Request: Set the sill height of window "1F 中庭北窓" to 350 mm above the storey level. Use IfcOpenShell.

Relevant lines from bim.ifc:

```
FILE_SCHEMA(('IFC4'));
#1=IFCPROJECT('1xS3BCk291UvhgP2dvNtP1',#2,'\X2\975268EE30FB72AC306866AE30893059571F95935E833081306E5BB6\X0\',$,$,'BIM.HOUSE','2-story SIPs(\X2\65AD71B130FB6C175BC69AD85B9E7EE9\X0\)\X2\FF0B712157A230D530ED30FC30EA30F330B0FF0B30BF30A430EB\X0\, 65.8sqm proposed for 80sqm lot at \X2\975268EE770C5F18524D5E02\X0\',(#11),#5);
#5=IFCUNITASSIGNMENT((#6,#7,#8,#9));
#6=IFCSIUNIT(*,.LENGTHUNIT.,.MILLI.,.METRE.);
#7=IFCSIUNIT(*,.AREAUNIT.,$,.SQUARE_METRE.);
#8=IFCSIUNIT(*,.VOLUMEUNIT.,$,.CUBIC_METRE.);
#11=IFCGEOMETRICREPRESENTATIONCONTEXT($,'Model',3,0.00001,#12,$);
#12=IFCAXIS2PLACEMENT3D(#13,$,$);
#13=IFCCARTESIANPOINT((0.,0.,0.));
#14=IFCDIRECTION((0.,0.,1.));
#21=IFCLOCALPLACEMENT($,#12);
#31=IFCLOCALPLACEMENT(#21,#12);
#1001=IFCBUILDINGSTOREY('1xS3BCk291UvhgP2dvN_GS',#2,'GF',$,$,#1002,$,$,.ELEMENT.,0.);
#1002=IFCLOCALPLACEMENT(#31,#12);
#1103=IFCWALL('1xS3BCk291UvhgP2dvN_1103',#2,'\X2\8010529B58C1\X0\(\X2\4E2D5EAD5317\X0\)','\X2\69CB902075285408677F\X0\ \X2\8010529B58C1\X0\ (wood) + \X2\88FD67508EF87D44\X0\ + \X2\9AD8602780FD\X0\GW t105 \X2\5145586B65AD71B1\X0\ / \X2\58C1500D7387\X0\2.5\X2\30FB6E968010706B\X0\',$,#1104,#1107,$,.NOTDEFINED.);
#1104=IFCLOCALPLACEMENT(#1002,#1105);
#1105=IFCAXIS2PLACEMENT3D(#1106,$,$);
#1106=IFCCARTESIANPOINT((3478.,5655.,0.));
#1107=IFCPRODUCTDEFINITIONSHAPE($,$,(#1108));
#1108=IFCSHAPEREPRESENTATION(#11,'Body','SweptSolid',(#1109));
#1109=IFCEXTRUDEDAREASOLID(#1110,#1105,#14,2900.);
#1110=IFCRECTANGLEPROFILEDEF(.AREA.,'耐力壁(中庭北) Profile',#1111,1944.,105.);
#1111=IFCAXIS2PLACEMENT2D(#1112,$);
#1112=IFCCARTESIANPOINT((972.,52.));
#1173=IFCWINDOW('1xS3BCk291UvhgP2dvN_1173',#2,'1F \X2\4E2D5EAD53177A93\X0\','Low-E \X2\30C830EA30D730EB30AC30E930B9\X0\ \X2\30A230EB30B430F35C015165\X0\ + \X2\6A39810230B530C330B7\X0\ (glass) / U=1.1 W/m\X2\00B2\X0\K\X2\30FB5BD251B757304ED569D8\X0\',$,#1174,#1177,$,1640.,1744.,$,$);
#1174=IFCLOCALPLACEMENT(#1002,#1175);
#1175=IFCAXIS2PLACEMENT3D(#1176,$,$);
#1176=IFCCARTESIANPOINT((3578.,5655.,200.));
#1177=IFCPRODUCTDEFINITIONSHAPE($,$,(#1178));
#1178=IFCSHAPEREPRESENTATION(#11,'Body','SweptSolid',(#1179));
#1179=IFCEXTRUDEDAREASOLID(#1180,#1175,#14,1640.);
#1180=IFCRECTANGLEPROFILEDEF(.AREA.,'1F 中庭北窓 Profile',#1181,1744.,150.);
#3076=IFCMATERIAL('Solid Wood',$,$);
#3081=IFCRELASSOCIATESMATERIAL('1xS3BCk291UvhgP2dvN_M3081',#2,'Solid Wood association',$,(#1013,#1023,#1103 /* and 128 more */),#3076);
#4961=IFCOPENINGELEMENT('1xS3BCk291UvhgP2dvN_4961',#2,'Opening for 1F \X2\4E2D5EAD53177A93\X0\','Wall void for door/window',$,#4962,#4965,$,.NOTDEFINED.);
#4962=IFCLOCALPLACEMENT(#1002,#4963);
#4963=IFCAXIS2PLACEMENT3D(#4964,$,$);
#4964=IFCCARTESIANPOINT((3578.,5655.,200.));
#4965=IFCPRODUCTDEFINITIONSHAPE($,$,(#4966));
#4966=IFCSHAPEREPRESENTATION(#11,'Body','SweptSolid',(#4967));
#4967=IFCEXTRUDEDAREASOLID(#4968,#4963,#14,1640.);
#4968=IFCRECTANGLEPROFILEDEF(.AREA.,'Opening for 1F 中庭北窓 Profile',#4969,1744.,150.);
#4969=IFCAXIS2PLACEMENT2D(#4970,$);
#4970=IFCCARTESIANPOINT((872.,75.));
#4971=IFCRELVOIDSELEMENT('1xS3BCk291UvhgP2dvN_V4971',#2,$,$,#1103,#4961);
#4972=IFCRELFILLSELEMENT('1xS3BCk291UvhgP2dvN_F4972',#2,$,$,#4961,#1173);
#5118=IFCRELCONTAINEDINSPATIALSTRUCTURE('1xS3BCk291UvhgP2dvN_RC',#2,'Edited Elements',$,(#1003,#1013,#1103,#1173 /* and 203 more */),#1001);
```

```python
import numpy as np
import ifcopenshell
import ifcopenshell.api.geometry
import ifcopenshell.geom
import ifcopenshell.util.element
import ifcopenshell.util.placement
import ifcopenshell.util.shape
import ifcopenshell.util.unit

model = ifcopenshell.open("bim.ifc")
unit_scale = ifcopenshell.util.unit.calculate_unit_scale(model)

window = model.by_guid("1xS3BCk291UvhgP2dvN_1173")
opening = window.FillsVoids[0].RelatingOpeningElement
storey = ifcopenshell.util.element.get_container(window, ifc_class="IfcBuildingStorey")
level = ifcopenshell.util.placement.get_local_placement(storey.ObjectPlacement)[2, 3]

# The opening's origin need not be at the sill, so measure its lowest point.
shape = ifcopenshell.geom.create_shape(ifcopenshell.geom.settings(), opening)
bottom = ifcopenshell.util.shape.get_shape_bottom_elevation(shape, shape.geometry) / unit_scale
dz = level + 350.0 - bottom

shift = np.array([0.0, 0.0, dz])
# The window is not placed relative to its opening, so move both.
for product in (opening, window):
    matrix = ifcopenshell.util.placement.get_local_placement(product.ObjectPlacement)
    matrix[:3, 3] += shift
    ifcopenshell.api.geometry.edit_object_placement(model, product=product, matrix=matrix, is_si=False)

print(f"moved by {dz * unit_scale:+.3f} m")

model.write("bim_edited.ifc")
```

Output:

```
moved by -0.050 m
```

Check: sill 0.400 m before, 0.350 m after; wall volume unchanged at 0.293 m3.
